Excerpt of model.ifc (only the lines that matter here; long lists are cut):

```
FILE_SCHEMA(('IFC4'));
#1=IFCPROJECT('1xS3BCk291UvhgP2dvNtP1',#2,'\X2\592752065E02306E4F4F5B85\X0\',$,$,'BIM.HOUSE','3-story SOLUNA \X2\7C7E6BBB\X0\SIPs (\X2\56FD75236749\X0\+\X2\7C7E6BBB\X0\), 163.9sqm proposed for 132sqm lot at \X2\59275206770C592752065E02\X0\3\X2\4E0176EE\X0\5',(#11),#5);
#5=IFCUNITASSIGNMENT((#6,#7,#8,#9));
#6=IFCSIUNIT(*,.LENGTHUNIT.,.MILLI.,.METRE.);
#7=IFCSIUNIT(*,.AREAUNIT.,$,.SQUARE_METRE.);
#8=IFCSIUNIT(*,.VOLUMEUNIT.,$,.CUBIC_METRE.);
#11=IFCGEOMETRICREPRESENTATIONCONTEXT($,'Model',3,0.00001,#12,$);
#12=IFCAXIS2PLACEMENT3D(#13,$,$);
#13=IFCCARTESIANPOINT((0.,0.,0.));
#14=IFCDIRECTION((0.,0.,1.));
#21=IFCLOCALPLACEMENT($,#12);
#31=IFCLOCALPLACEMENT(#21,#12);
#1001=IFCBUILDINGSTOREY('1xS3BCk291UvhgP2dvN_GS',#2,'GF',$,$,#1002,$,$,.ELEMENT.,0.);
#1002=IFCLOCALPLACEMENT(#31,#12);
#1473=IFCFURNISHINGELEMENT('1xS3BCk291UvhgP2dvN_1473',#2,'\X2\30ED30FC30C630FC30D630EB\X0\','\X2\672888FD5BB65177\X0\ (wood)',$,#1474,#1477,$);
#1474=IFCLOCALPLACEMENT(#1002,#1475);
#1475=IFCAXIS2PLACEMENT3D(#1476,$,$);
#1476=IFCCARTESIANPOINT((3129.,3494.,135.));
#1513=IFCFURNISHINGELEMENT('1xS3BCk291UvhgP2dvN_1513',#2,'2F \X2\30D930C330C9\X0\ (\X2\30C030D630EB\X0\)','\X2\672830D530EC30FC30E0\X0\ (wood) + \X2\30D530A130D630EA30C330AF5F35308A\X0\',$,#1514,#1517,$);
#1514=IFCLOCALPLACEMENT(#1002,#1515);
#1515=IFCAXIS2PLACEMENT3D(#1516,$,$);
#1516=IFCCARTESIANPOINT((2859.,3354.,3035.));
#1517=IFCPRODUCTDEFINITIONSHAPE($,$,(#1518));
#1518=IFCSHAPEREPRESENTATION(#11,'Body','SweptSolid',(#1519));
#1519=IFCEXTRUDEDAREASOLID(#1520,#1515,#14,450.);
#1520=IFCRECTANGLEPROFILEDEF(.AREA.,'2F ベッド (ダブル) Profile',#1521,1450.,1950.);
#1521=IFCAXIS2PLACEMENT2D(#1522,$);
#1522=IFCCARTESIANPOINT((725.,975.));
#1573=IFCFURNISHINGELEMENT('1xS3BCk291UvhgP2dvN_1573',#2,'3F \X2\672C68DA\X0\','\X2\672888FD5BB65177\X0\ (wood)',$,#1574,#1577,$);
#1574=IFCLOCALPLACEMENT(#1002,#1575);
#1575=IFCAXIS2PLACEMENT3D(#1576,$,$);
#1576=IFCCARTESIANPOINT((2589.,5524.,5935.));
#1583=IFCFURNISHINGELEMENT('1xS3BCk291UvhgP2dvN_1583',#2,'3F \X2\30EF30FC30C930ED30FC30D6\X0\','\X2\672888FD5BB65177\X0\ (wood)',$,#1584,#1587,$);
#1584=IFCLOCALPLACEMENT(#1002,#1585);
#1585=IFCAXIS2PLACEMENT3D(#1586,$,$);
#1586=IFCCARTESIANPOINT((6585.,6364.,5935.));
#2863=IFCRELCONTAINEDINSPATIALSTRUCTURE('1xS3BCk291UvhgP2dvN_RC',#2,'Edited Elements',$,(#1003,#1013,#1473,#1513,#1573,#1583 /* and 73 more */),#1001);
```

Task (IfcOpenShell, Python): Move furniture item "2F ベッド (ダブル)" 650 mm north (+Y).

```python
import ifcopenshell
import ifcopenshell.api.geometry
import ifcopenshell.util.placement
import ifcopenshell.util.unit

model = ifcopenshell.open("model.ifc")
unit_scale = ifcopenshell.util.unit.calculate_unit_scale(model)

item = model.by_id(1513)
matrix = ifcopenshell.util.placement.get_local_placement(item.ObjectPlacement)
matrix[1, 3] += 0.65 / unit_scale
ifcopenshell.api.geometry.edit_object_placement(model, product=item, matrix=matrix, is_si=False)

print(ifcopenshell.util.placement.get_local_placement(item.ObjectPlacement).round(3) + 0.0)

model.write("model-out.ifc")
```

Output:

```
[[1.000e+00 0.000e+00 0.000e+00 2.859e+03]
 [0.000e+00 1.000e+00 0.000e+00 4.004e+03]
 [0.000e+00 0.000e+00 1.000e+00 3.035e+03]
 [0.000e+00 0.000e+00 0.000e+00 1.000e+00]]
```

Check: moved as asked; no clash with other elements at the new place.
